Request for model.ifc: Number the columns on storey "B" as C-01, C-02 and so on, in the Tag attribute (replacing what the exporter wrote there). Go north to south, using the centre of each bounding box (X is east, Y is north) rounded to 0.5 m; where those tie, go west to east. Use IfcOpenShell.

First a look at what the model holds.

```python
import ifcopenshell
import ifcopenshell.util.element
import ifcopenshell.util.placement

model = ifcopenshell.open("model.ifc")
print(model.schema)
storey = next(s for s in model.by_type("IfcBuildingStorey") if s.Name == "B")
columns = [e for e in ifcopenshell.util.element.get_decomposition(storey) if e.is_a("IfcColumn")]
for e in sorted(columns, key=lambda e: e.id()):
    origin = ifcopenshell.util.placement.get_local_placement(e.ObjectPlacement)[:3, 3]
    print(e.id(), e.Tag, e.Name, origin.round(2) + 0.0, sep=" | ")
```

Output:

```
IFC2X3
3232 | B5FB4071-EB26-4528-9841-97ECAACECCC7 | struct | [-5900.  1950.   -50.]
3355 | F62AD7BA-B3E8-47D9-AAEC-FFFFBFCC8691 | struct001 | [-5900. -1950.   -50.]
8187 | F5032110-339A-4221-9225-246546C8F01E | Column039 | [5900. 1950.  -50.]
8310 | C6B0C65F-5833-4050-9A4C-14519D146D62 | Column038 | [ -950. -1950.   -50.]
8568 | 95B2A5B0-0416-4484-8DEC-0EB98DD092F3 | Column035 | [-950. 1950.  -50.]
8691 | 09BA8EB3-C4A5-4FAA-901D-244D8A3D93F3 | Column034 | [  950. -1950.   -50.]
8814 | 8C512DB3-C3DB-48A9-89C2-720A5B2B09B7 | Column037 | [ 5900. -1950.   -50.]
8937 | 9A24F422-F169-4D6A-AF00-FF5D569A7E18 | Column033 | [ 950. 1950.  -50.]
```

```python
import ifcopenshell
import ifcopenshell.geom
import ifcopenshell.util.element
import ifcopenshell.util.shape

model = ifcopenshell.open("model.ifc")
settings = ifcopenshell.geom.settings()
settings.set("use-world-coords", True)


def centre(element):
    shape = ifcopenshell.geom.create_shape(settings, element)
    return ifcopenshell.util.shape.get_bbox_centroid(shape.geometry)


storey = next(s for s in model.by_type("IfcBuildingStorey") if s.Name == "B")
columns = [e for e in ifcopenshell.util.element.get_decomposition(storey) if e.is_a("IfcColumn")]

# Insertion points can sit at a corner or the storey origin, so sort by the geometry (in metres).
centres = {e: centre(e) for e in columns}
columns.sort(key=lambda e: (-round(centres[e][1] / 0.5), centres[e][0]))

for i, e in enumerate(columns, start=1):
    number = f"C-{i:02d}"
    e.Tag = number
    print(e.id(), number)

model.write("model_updated.ifc")
```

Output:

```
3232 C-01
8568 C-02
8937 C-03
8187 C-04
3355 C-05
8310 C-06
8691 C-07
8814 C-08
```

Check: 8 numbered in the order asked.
